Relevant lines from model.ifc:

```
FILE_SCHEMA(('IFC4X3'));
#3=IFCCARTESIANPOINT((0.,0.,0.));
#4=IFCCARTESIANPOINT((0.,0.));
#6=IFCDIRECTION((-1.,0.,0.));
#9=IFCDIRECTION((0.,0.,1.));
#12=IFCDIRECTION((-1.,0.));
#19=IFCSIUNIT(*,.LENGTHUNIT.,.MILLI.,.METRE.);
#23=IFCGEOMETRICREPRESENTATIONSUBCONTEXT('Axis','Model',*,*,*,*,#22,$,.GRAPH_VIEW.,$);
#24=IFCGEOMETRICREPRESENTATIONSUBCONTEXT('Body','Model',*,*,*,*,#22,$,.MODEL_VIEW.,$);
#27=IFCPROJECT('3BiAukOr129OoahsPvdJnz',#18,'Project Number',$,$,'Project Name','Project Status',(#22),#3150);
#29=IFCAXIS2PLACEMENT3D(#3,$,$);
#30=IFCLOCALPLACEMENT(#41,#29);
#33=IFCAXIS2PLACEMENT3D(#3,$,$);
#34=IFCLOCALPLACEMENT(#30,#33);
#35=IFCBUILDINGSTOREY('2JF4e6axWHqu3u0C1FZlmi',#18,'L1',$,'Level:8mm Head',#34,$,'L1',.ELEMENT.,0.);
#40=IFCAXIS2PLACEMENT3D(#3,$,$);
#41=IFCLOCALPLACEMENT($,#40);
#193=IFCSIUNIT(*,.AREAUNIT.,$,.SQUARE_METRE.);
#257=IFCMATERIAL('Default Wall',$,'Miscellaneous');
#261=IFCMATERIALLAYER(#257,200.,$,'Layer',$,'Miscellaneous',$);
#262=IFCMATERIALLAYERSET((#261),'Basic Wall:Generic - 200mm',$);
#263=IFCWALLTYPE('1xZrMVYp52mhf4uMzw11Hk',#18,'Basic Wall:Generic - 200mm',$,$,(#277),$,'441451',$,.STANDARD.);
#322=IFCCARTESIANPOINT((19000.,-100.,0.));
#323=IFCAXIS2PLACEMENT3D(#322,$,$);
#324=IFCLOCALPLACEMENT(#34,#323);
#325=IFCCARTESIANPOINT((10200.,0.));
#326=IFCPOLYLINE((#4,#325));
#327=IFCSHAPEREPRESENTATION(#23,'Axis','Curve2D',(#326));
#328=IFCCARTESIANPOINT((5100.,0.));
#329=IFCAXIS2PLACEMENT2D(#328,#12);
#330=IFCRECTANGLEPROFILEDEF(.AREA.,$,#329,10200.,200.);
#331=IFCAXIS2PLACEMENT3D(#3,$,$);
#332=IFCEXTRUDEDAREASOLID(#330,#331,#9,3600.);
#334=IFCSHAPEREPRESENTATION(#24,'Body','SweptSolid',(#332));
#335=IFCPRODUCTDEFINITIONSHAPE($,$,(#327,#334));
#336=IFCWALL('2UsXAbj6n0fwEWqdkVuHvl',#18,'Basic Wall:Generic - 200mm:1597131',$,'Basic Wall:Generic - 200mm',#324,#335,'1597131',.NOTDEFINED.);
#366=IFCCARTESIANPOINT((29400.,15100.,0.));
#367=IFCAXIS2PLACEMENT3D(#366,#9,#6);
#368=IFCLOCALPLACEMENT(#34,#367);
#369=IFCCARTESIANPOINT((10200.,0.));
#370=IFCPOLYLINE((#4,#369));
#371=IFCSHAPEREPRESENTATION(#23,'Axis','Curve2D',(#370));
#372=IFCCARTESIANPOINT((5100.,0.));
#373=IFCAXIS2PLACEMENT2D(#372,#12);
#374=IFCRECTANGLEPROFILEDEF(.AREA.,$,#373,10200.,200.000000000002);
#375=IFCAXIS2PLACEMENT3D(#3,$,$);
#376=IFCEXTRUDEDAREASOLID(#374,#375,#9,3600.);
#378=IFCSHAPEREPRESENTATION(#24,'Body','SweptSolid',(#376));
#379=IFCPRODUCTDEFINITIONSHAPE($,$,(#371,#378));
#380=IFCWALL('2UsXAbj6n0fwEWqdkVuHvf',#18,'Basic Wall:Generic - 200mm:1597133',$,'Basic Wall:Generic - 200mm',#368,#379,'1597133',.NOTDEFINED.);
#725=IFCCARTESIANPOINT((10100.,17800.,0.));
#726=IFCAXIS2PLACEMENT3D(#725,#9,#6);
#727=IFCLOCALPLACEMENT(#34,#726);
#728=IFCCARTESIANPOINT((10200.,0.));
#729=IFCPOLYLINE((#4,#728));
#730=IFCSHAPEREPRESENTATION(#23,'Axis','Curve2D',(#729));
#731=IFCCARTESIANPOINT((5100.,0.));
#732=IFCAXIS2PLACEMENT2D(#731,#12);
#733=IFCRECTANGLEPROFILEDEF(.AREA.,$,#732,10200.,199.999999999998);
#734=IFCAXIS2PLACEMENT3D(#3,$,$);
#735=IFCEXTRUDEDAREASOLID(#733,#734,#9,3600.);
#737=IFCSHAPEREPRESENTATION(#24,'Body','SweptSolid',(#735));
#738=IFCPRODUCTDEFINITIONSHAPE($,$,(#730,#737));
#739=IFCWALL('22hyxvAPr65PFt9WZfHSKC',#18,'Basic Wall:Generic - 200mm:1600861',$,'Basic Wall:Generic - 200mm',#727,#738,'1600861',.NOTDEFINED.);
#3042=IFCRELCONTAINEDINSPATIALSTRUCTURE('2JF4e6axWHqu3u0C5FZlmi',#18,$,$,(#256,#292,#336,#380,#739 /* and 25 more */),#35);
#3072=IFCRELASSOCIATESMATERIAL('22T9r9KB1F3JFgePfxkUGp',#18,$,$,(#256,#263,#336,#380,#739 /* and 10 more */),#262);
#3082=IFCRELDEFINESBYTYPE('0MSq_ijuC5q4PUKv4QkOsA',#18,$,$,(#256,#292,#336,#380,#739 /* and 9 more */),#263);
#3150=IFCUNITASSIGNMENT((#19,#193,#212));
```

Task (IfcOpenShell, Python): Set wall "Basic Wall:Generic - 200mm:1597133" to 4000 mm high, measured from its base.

```python
import ifcopenshell
import ifcopenshell.geom
import ifcopenshell.util.representation
import ifcopenshell.util.shape

model = ifcopenshell.open("model.ifc")
settings = ifcopenshell.geom.settings()


def volume(element):
    """Net volume in cubic metres, openings subtracted."""
    shape = ifcopenshell.geom.create_shape(settings, element)
    return ifcopenshell.util.shape.get_volume(shape.geometry)


wall = model.by_id(380)
before = volume(wall)

body = ifcopenshell.util.representation.get_representation(wall, "Model", "Body")
solid = body.Items[0]
old_height = solid.Depth
solid.Depth = 4000.0
after = volume(wall)

print(f"height {old_height:g} -> {solid.Depth:g}, volume {before:.3f} -> {after:.3f} m3")

model.write("model_edited.ifc")
```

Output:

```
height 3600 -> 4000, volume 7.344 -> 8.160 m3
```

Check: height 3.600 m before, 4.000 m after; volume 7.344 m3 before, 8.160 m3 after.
